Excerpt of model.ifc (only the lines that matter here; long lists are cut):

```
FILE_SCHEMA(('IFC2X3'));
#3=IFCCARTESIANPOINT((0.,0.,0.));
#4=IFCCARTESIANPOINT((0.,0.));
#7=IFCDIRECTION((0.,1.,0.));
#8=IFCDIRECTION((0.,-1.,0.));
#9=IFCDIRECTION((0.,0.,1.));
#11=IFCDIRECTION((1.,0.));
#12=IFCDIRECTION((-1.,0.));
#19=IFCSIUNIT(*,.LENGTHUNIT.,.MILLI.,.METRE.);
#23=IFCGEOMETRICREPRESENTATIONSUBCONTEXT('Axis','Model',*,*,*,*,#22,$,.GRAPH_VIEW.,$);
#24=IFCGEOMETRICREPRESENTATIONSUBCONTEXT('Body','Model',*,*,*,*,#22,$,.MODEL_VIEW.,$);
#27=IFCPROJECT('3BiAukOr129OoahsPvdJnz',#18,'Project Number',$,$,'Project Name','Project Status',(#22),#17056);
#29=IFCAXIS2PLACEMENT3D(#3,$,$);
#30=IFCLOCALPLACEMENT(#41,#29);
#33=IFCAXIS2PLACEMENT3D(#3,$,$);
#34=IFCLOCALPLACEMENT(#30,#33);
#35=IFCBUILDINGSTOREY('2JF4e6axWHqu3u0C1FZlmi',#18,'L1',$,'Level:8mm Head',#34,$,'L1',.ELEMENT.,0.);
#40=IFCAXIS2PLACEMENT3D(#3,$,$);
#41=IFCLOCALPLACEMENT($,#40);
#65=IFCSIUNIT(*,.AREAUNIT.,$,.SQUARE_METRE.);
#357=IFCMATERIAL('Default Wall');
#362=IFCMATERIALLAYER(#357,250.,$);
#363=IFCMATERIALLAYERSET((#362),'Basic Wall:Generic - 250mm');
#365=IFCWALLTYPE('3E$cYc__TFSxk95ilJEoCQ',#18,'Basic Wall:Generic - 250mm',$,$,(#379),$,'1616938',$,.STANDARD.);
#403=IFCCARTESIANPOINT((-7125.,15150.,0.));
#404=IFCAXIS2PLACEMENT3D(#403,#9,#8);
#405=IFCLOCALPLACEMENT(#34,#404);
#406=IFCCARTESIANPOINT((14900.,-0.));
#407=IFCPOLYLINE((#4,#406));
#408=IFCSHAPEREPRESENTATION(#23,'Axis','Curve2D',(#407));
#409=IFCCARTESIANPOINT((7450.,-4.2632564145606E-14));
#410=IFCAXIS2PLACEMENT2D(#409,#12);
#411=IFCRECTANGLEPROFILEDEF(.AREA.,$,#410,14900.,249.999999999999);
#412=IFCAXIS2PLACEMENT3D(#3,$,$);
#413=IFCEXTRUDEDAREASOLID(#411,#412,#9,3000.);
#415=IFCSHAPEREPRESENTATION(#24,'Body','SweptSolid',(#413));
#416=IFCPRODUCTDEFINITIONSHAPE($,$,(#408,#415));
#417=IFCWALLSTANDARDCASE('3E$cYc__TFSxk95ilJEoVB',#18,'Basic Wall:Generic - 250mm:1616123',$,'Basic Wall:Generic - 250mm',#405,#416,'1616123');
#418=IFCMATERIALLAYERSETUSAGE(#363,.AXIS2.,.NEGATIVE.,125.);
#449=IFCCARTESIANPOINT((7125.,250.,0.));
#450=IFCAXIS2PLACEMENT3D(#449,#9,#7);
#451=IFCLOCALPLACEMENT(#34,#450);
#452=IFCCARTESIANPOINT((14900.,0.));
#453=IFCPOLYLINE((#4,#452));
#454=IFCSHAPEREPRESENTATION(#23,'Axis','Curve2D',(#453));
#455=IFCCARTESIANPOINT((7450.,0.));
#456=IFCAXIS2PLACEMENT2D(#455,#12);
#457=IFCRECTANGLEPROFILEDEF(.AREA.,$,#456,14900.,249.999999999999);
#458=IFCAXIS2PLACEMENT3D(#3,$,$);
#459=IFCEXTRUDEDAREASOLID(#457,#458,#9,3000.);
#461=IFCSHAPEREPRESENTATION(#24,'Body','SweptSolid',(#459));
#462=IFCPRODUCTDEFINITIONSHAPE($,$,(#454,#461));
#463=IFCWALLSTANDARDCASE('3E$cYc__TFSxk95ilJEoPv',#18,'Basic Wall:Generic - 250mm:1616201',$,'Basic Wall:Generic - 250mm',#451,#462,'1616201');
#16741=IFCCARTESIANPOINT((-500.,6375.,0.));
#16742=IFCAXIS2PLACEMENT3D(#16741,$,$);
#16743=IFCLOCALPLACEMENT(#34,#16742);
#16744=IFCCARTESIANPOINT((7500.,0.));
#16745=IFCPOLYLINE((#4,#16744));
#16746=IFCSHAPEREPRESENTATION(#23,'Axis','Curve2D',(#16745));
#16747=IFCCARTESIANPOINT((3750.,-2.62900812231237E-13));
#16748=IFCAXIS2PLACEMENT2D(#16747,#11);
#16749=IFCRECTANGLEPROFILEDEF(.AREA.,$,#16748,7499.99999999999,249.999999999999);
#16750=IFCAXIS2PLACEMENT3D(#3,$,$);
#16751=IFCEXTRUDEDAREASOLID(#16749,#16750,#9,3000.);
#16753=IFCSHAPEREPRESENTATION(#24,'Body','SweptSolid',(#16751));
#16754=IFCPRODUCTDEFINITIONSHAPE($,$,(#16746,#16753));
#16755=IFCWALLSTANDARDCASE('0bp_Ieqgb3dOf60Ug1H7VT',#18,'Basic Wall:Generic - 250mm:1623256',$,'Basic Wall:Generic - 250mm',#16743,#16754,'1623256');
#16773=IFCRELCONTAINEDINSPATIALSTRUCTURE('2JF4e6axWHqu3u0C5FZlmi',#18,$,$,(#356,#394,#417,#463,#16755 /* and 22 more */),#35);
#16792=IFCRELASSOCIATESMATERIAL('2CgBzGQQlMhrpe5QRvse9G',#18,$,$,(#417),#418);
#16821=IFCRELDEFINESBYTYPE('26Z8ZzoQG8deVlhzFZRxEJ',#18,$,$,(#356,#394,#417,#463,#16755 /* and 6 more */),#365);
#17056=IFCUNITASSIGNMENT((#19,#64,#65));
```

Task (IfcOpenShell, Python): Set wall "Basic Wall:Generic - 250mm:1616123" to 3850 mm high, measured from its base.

```python
import ifcopenshell
import ifcopenshell.geom
import ifcopenshell.util.representation
import ifcopenshell.util.shape

model = ifcopenshell.open("model.ifc")
settings = ifcopenshell.geom.settings()


def volume(element):
    """Net volume in cubic metres, openings subtracted."""
    shape = ifcopenshell.geom.create_shape(settings, element)
    return ifcopenshell.util.shape.get_volume(shape.geometry)


wall = model.by_guid("3E$cYc__TFSxk95ilJEoVB")
before = volume(wall)

body = ifcopenshell.util.representation.get_representation(wall, "Model", "Body")
solid = body.Items[0]
old_height = solid.Depth
solid.Depth = 3850.0
after = volume(wall)

print(f"height {old_height:g} -> {solid.Depth:g}, volume {before:.3f} -> {after:.3f} m3")

model.write("model_edited.ifc")
```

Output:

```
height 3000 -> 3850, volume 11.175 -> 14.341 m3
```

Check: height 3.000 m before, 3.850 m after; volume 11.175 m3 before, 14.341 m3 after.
